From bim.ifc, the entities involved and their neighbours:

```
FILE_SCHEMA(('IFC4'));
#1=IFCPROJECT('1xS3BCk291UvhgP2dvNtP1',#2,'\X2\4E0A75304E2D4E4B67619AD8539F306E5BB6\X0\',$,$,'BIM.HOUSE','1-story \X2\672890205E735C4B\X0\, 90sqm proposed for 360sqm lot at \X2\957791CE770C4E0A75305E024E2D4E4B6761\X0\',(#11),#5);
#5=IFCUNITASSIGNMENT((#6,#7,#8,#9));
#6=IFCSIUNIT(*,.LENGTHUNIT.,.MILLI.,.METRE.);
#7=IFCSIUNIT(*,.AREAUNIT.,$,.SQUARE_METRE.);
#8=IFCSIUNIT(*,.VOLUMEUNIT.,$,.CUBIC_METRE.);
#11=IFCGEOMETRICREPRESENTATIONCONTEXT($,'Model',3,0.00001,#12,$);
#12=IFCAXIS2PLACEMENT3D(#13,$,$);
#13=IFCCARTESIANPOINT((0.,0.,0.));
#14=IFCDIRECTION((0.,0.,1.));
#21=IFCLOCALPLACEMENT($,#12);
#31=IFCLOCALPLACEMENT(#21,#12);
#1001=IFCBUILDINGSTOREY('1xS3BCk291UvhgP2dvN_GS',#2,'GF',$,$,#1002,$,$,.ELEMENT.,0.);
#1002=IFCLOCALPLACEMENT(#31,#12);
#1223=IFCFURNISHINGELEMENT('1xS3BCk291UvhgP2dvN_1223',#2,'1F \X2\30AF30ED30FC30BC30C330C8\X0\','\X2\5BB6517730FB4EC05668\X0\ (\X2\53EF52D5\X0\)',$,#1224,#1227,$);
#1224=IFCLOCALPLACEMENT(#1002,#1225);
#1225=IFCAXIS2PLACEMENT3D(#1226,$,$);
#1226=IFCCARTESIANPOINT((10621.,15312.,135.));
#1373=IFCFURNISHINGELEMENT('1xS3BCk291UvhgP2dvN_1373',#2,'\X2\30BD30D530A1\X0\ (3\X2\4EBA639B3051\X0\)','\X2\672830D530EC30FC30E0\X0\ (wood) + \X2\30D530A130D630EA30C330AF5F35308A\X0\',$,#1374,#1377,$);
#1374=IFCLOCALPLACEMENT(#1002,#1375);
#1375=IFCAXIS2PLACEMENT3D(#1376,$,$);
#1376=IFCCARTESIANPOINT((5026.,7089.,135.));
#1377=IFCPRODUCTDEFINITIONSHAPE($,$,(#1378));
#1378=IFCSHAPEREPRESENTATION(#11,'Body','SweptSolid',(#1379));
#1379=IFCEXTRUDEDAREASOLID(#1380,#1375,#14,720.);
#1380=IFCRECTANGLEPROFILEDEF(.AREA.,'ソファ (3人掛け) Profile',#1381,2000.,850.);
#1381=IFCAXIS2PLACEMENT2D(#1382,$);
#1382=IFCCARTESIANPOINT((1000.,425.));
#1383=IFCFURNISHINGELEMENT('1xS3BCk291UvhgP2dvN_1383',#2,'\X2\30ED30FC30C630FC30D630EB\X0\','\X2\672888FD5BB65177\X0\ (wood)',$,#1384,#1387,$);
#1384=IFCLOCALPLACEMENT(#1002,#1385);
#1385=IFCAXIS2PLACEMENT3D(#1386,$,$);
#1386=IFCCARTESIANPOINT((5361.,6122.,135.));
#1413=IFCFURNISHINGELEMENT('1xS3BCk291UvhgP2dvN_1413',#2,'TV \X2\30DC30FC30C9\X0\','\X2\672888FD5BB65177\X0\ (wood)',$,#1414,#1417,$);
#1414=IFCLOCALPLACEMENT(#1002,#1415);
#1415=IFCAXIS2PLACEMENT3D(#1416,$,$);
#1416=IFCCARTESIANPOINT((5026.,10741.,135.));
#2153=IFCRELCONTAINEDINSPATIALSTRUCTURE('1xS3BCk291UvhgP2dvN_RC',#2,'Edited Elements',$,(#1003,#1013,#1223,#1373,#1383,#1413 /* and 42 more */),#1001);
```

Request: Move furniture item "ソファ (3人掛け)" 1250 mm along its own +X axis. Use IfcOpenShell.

```python
import ifcopenshell
import ifcopenshell.api.geometry
import ifcopenshell.util.placement
import ifcopenshell.util.unit

model = ifcopenshell.open("bim.ifc")
unit_scale = ifcopenshell.util.unit.calculate_unit_scale(model)

item = model.by_guid("1xS3BCk291UvhgP2dvN_1373")
matrix = ifcopenshell.util.placement.get_local_placement(item.ObjectPlacement)
matrix[:3, 3] += matrix[:3, 0] * 1.25 / unit_scale
ifcopenshell.api.geometry.edit_object_placement(model, product=item, matrix=matrix, is_si=False)

print(ifcopenshell.util.placement.get_local_placement(item.ObjectPlacement).round(3) + 0.0)

model.write("bim_edited.ifc")
```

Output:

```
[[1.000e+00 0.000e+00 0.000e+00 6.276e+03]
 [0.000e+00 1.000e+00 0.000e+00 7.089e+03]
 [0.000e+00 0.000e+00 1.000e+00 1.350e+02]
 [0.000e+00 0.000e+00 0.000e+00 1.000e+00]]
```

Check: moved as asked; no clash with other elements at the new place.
